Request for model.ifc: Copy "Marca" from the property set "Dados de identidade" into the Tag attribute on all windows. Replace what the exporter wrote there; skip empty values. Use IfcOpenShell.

First a look at what the model holds.

```python
import ifcopenshell
import ifcopenshell.util.element

model = ifcopenshell.open("model.ifc")
print(model.schema)
windows = model.by_type("IfcWindow")
print(len(windows), "windows")
for e in windows[:8]:
    source = ifcopenshell.util.element.get_pset(e, "Dados de identidade", "Marca")
    target = e.Tag
    print(e.id(), repr(source), repr(target), sep=" | ")
```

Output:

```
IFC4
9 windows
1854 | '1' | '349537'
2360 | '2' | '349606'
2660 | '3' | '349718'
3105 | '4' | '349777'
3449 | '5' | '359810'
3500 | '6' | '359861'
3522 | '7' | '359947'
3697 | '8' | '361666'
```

```python
import ifcopenshell
import ifcopenshell.util.element

model = ifcopenshell.open("model.ifc")

count = 0
for e in model.by_type("IfcWindow"):
    value = ifcopenshell.util.element.get_pset(e, "Dados de identidade", "Marca")
    current = e.Tag
    if not value or not value.strip() or current == value:
        continue
    e.Tag = value
    count += 1

print(count, "windows updated")

model.write("model_v2.ifc")
```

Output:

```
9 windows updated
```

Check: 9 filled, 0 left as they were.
